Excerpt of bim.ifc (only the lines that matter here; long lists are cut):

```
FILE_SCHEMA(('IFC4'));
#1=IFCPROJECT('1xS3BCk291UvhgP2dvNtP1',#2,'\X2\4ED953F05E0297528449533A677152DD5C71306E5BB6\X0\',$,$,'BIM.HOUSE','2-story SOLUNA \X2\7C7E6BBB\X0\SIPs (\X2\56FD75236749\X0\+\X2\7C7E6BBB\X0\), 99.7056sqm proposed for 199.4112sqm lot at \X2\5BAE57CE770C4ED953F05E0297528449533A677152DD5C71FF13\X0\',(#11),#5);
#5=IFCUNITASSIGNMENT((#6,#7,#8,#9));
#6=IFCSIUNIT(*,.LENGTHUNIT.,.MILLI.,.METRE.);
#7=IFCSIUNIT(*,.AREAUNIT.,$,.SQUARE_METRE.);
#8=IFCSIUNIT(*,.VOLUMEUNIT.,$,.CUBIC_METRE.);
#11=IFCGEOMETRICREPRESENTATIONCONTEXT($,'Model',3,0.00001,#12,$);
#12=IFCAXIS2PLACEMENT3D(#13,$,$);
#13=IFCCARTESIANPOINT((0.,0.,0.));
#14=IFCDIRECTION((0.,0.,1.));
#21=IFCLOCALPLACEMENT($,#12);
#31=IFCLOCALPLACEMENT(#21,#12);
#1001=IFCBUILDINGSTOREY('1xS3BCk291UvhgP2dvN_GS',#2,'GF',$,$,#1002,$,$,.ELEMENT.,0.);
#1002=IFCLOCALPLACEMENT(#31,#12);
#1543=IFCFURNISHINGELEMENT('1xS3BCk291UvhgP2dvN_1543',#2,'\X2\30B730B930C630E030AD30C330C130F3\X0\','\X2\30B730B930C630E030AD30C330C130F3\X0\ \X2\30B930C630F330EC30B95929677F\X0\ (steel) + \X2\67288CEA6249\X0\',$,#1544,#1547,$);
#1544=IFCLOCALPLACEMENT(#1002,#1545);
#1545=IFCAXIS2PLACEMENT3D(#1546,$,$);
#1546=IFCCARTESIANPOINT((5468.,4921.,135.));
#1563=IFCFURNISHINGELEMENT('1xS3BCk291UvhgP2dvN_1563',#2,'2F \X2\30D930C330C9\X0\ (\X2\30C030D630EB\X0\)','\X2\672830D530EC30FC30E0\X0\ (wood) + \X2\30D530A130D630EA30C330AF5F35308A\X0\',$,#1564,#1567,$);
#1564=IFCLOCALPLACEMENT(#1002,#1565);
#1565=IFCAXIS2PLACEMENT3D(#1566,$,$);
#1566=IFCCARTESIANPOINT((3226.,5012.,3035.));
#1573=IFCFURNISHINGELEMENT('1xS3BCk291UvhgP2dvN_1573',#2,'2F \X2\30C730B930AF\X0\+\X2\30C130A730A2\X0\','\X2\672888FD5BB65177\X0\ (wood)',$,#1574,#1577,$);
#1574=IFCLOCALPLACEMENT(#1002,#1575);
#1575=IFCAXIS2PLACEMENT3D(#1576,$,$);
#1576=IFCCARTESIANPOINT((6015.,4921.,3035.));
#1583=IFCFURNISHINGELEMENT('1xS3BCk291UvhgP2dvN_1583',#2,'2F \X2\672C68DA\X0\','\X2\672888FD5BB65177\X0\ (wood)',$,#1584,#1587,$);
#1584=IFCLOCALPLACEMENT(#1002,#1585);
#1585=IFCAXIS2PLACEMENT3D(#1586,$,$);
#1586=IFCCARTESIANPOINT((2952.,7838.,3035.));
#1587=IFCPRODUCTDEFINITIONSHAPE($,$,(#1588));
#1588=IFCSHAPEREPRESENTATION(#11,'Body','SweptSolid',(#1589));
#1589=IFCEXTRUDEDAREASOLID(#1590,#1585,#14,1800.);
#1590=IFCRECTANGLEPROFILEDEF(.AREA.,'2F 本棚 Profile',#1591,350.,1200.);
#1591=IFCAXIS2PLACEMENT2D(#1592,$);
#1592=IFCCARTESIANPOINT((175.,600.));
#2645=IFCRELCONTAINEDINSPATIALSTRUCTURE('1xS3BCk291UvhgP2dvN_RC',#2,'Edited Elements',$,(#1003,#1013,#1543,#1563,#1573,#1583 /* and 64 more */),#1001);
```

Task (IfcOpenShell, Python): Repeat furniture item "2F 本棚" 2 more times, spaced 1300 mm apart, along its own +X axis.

```python
import ifcopenshell
import ifcopenshell.api.geometry
import ifcopenshell.api.root
import ifcopenshell.util.element
import ifcopenshell.util.placement

model = ifcopenshell.open("bim.ifc")


def reuse_history(source, copy):
    """copy_class also copies each property set's owner history, people and application; keep the originals."""
    for rel in copy.IsDefinedBy:
        if rel.is_a("IfcRelDefinesByProperties") and (history := rel.RelatingPropertyDefinition.OwnerHistory):
            rel.RelatingPropertyDefinition.OwnerHistory = source.OwnerHistory
            ifcopenshell.util.element.remove_deep2(model, history)


source = model.by_guid("1xS3BCk291UvhgP2dvN_1583")
base = ifcopenshell.util.placement.get_local_placement(source.ObjectPlacement)
step = base[:3, 0] * 1300.0

for i in range(1, 3):
    copy = ifcopenshell.api.root.copy_class(model, product=source)
    copy.Representation = ifcopenshell.util.element.copy_deep(
        model, source.Representation, exclude=["IfcGeometricRepresentationContext", "IfcRepresentationMap"]
    )
    reuse_history(source, copy)
    matrix = base.copy()
    matrix[:3, 3] += i * step
    print("added at", matrix[:3, 3].round(3) + 0.0)
    ifcopenshell.api.geometry.edit_object_placement(model, product=copy, matrix=matrix, is_si=False)

model.write("bim_edited.ifc")
```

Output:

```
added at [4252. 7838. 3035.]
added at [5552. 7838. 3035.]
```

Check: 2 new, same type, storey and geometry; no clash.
